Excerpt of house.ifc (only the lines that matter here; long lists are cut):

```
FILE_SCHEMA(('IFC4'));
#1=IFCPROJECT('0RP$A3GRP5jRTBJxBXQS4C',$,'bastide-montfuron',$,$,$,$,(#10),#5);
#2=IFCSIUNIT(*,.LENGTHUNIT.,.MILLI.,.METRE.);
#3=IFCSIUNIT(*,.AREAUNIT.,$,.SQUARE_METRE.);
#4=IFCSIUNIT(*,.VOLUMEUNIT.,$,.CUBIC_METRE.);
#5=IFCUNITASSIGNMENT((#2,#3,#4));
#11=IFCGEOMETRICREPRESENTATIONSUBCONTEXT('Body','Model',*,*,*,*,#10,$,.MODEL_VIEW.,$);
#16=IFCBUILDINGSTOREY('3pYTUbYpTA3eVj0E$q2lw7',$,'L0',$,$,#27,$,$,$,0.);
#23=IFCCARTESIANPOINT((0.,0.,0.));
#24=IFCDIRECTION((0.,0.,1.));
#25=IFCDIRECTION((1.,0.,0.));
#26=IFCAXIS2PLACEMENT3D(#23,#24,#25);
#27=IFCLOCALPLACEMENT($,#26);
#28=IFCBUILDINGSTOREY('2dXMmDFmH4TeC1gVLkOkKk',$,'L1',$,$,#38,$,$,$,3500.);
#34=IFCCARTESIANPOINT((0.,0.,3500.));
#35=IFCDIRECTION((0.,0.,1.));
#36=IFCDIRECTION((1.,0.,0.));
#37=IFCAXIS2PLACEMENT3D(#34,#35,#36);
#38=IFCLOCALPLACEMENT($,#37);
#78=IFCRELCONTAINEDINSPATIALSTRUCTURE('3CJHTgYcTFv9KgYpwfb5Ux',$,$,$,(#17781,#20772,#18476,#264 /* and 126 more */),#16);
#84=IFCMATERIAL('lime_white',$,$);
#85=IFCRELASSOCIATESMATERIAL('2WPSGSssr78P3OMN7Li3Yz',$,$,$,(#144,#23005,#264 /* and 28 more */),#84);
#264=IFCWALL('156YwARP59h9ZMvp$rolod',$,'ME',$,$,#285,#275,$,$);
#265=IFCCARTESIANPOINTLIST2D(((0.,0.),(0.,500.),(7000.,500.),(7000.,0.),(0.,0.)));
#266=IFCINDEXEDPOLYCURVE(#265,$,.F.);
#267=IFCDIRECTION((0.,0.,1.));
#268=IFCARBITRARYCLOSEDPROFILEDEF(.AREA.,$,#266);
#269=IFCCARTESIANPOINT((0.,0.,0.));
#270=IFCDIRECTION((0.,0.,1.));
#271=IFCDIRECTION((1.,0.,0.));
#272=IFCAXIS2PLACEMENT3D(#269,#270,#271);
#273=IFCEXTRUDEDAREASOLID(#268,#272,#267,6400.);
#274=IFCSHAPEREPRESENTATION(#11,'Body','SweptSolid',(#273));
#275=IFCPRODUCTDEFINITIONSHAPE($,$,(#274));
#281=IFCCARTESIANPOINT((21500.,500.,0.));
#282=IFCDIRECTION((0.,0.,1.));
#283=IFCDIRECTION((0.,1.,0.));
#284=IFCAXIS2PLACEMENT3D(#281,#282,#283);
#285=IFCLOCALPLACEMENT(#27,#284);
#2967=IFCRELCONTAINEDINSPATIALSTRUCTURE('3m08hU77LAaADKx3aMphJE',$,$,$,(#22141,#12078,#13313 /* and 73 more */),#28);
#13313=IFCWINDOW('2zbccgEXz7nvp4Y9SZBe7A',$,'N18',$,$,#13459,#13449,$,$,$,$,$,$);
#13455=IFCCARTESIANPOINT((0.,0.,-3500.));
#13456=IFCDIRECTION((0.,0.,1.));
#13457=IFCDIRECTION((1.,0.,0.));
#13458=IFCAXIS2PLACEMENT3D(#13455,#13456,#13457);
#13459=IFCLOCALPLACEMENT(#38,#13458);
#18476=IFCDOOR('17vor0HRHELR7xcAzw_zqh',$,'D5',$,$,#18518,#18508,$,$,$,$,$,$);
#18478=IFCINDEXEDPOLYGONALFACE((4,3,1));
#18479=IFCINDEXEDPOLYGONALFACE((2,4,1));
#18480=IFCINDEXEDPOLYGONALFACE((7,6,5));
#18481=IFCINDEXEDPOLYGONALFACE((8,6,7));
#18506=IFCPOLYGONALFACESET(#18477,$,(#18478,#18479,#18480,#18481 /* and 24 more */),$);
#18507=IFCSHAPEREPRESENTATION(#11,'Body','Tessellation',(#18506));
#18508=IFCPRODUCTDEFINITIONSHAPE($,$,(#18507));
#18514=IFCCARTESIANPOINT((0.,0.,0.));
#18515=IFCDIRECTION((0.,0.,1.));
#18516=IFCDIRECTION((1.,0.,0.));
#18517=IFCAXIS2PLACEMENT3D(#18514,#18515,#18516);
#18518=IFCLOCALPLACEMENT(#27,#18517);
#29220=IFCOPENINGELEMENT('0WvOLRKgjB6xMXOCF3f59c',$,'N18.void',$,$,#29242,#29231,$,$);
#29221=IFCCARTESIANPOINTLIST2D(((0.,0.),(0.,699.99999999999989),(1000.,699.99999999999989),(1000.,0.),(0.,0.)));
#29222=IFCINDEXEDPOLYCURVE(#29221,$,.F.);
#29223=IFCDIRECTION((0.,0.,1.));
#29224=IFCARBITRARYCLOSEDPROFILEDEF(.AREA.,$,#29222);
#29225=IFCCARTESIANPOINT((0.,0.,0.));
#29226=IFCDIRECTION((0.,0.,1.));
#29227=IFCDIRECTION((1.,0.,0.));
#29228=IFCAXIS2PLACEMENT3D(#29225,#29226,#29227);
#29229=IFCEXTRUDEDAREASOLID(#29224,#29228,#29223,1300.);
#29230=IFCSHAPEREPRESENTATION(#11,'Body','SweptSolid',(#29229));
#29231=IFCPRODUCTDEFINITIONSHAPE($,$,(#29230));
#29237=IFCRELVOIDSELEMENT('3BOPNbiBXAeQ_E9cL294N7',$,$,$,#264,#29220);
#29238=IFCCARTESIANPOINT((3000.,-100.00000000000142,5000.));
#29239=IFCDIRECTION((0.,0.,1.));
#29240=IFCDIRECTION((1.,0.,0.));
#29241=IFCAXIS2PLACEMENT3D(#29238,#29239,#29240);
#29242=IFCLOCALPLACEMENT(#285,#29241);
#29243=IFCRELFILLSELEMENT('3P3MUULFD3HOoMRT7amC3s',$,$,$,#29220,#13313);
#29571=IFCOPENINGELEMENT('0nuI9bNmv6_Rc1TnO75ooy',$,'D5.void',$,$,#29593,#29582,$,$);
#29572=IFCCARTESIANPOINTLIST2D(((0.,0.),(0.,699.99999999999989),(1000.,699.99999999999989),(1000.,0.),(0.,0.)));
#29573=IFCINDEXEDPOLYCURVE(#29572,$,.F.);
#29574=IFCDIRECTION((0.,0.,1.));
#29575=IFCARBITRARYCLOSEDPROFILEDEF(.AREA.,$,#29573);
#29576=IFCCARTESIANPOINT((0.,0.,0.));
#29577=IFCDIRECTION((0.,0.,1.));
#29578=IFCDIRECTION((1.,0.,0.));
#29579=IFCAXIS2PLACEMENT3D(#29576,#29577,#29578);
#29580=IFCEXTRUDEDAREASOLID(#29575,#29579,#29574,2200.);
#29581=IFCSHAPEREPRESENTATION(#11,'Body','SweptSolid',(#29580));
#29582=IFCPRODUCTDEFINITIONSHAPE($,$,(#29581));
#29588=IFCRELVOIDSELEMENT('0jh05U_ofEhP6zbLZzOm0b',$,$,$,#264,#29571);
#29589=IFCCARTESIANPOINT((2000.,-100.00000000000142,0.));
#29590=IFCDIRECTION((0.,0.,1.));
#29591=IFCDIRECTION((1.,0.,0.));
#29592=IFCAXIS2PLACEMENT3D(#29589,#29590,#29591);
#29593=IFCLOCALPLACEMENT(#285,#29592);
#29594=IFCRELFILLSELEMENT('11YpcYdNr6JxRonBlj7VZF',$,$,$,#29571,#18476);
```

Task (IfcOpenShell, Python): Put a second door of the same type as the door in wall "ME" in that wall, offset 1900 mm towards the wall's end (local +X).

```python
import ifcopenshell
import ifcopenshell.api.feature
import ifcopenshell.api.geometry
import ifcopenshell.api.root
import ifcopenshell.geom
import ifcopenshell.util.element
import ifcopenshell.util.placement
import ifcopenshell.util.shape
import ifcopenshell.util.unit

model = ifcopenshell.open("house.ifc")
unit_scale = ifcopenshell.util.unit.calculate_unit_scale(model)
settings = ifcopenshell.geom.settings()


def volume(element):
    """Net volume in cubic metres, openings subtracted."""
    shape = ifcopenshell.geom.create_shape(settings, element)
    return ifcopenshell.util.shape.get_volume(shape.geometry)


door = model.by_guid("17vor0HRHELR7xcAzw_zqh")
opening = door.FillsVoids[0].RelatingOpeningElement
wall = opening.VoidsElements[0].RelatingBuildingElement
before = volume(wall)
shift = ifcopenshell.util.placement.get_local_placement(wall.ObjectPlacement)[:3, 0] * 1.9 / unit_scale

# copy_class copies the void relationship, type, container and properties, but no geometry.
new_opening = ifcopenshell.api.root.copy_class(model, product=opening)
new_opening.Representation = ifcopenshell.util.element.copy_deep(
    model, opening.Representation, exclude=["IfcGeometricRepresentationContext", "IfcRepresentationMap"]
)
new_door = ifcopenshell.api.root.copy_class(model, product=door)
new_door.Representation = ifcopenshell.util.element.copy_deep(
    model, door.Representation, exclude=["IfcGeometricRepresentationContext", "IfcRepresentationMap"]
)
ifcopenshell.api.feature.add_filling(model, opening=new_opening, element=new_door)

for old, new in ((opening, new_opening), (door, new_door)):
    matrix = ifcopenshell.util.placement.get_local_placement(old.ObjectPlacement)
    matrix[:3, 3] += shift
    ifcopenshell.api.geometry.edit_object_placement(model, product=new, matrix=matrix, is_si=False)

after = volume(wall)

print(f"wall volume {before:.3f} -> {after:.3f} m3")

model.write("house_rev.ifc")
```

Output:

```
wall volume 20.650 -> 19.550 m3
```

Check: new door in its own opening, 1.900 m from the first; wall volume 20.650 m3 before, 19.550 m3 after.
